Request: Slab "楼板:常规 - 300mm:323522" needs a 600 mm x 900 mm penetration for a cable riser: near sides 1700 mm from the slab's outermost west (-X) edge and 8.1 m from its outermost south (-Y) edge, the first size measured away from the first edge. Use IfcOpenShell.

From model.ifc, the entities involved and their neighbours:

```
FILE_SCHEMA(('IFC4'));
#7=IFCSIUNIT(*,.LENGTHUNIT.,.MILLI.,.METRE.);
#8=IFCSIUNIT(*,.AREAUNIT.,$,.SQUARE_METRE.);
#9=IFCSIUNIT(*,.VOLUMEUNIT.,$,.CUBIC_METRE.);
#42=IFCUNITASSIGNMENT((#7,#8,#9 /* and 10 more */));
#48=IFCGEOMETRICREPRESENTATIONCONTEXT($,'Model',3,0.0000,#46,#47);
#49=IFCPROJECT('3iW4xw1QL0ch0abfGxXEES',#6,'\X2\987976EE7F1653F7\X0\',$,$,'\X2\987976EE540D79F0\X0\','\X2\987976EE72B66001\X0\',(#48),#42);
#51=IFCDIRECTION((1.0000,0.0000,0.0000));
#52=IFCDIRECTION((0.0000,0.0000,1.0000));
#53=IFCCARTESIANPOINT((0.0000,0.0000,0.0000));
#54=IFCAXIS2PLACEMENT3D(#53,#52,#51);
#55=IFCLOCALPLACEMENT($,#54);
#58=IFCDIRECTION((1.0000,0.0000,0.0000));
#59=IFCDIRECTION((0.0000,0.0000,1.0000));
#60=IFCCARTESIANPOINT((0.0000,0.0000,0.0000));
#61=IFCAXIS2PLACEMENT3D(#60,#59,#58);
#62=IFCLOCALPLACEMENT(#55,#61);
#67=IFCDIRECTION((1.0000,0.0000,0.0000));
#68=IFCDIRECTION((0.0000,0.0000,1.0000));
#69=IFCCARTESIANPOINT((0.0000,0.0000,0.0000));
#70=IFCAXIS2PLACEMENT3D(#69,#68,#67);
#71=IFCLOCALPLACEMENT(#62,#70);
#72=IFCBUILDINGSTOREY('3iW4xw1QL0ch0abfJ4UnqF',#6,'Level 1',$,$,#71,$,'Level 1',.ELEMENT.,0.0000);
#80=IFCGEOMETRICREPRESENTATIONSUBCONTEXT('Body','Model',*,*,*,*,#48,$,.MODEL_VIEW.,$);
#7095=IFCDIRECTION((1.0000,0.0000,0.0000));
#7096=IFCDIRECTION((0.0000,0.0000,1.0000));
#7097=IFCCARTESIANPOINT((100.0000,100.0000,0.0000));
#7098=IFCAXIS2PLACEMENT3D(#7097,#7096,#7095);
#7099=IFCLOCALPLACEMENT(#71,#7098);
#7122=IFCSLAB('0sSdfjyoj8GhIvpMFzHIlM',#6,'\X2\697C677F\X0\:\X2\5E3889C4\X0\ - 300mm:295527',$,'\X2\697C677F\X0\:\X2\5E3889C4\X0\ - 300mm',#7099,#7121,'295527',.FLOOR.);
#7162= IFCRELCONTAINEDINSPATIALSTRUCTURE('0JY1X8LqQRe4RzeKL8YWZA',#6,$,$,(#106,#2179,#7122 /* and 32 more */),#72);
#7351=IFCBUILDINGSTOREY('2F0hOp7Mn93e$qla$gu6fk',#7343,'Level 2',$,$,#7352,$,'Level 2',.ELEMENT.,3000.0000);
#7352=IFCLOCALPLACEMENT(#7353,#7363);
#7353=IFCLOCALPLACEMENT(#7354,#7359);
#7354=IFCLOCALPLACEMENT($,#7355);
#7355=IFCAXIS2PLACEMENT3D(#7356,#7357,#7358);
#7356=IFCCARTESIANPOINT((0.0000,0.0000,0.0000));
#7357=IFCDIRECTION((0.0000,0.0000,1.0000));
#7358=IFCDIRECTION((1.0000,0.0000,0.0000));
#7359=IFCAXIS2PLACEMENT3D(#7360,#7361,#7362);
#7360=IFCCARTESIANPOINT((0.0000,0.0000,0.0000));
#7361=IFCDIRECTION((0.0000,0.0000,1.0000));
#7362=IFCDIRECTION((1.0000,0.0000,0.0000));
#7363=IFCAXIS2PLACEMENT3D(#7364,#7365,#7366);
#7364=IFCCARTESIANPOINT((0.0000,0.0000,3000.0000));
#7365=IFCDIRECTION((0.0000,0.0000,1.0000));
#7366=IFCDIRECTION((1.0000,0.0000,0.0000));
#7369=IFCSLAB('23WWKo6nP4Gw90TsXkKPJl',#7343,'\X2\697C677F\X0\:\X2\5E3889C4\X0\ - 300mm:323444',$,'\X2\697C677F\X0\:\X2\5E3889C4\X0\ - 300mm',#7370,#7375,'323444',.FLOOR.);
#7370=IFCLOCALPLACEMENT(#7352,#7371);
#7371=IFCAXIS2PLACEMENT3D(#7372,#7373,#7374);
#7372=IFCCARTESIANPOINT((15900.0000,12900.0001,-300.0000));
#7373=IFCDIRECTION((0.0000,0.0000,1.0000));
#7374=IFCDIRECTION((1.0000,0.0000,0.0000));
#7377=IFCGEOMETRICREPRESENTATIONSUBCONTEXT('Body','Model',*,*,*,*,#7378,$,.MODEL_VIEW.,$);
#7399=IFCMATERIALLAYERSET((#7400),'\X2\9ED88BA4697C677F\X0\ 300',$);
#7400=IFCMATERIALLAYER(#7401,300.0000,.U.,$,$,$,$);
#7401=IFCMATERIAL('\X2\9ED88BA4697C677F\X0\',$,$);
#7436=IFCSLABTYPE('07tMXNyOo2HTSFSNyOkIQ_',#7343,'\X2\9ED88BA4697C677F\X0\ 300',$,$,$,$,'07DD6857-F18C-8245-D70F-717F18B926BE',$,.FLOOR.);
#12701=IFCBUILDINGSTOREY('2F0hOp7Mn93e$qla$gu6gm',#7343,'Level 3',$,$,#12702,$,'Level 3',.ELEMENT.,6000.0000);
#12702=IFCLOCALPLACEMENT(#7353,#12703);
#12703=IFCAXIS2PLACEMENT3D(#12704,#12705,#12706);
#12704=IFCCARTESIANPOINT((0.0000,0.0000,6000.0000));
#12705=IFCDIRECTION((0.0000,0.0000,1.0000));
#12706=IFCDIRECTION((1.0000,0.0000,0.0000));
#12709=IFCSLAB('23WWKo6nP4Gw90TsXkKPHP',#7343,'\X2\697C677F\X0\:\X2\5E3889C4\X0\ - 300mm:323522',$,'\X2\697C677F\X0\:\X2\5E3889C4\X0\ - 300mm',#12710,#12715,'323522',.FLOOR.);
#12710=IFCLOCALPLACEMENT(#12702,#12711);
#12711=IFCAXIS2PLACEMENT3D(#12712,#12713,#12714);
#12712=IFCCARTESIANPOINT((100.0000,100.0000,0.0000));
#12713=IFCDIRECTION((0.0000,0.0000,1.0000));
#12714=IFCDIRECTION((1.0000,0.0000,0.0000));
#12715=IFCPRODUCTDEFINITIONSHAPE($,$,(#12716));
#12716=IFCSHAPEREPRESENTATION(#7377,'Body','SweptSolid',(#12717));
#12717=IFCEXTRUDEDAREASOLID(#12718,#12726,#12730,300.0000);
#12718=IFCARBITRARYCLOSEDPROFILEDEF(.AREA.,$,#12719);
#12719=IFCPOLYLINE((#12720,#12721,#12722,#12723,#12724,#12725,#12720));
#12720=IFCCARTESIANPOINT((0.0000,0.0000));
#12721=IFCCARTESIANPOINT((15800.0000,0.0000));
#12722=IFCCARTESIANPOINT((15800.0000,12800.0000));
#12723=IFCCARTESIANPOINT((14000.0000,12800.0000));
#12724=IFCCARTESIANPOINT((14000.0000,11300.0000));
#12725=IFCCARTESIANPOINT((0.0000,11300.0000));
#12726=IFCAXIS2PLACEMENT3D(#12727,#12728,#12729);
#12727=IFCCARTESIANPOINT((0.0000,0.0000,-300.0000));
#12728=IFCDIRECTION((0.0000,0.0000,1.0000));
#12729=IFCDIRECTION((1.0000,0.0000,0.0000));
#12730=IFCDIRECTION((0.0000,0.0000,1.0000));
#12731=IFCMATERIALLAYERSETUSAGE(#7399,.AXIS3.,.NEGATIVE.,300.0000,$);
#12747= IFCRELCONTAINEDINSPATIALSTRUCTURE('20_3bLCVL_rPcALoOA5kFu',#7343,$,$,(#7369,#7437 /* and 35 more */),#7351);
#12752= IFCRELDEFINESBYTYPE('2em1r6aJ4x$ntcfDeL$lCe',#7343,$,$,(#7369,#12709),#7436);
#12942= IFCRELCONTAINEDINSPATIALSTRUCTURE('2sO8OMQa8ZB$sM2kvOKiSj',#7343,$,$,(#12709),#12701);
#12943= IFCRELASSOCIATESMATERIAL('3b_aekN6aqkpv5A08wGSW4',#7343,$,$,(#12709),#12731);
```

```python
import numpy as np
import ifcopenshell
import ifcopenshell.api.feature
import ifcopenshell.api.geometry
import ifcopenshell.api.root
import ifcopenshell.geom
import ifcopenshell.util.placement
import ifcopenshell.util.representation
import ifcopenshell.util.shape
import ifcopenshell.util.unit

model = ifcopenshell.open("model.ifc")
unit_scale = ifcopenshell.util.unit.calculate_unit_scale(model)
settings = ifcopenshell.geom.settings()


def volume(element):
    """Net volume in cubic metres, openings subtracted."""
    shape = ifcopenshell.geom.create_shape(settings, element)
    return ifcopenshell.util.shape.get_volume(shape.geometry)


slab = model.by_id(12709)
before = volume(slab)

# Extent in the slab's own axes, in metres. The edges named are its -X and -Y sides.
slab_shape = ifcopenshell.geom.create_shape(settings, slab)
vertices = ifcopenshell.util.shape.get_vertices(slab_shape.geometry)
x_min, y_min, bottom = vertices.min(axis=0)
top = vertices[:, 2].max()

opening = ifcopenshell.api.root.create_entity(model, ifc_class="IfcOpeningElement", name="Cable riser opening", predefined_type="OPENING")
context = ifcopenshell.util.representation.get_context(model, "Model", "Body", "MODEL_VIEW")
width, depth = 0.6, 0.9
outline = [(0.0, 0.0), (width, 0.0), (width, depth), (0.0, depth), (0.0, 0.0)]
# Overshoot both faces by 50 mm so the cut is clean.
shape = ifcopenshell.api.geometry.add_slab_representation(
    model, context=context, depth=top - bottom + 0.1, polyline=outline
)
ifcopenshell.api.geometry.assign_representation(model, product=opening, representation=shape)

matrix = ifcopenshell.util.placement.get_local_placement(slab.ObjectPlacement)
matrix[:, 3] = matrix @ np.append(np.array([x_min + 1.7, y_min + 8.1, bottom - 0.05]) / unit_scale, 1.0)
ifcopenshell.api.geometry.edit_object_placement(model, product=opening, matrix=matrix, is_si=False)
ifcopenshell.api.feature.add_feature(model, feature=opening, element=slab)

after = volume(slab)

print(f"slab volume {before:.3f} -> {after:.3f} m3")

model.write("model_updated.ifc")
```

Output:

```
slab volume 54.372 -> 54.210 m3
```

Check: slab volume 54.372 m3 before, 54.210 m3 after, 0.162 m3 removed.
